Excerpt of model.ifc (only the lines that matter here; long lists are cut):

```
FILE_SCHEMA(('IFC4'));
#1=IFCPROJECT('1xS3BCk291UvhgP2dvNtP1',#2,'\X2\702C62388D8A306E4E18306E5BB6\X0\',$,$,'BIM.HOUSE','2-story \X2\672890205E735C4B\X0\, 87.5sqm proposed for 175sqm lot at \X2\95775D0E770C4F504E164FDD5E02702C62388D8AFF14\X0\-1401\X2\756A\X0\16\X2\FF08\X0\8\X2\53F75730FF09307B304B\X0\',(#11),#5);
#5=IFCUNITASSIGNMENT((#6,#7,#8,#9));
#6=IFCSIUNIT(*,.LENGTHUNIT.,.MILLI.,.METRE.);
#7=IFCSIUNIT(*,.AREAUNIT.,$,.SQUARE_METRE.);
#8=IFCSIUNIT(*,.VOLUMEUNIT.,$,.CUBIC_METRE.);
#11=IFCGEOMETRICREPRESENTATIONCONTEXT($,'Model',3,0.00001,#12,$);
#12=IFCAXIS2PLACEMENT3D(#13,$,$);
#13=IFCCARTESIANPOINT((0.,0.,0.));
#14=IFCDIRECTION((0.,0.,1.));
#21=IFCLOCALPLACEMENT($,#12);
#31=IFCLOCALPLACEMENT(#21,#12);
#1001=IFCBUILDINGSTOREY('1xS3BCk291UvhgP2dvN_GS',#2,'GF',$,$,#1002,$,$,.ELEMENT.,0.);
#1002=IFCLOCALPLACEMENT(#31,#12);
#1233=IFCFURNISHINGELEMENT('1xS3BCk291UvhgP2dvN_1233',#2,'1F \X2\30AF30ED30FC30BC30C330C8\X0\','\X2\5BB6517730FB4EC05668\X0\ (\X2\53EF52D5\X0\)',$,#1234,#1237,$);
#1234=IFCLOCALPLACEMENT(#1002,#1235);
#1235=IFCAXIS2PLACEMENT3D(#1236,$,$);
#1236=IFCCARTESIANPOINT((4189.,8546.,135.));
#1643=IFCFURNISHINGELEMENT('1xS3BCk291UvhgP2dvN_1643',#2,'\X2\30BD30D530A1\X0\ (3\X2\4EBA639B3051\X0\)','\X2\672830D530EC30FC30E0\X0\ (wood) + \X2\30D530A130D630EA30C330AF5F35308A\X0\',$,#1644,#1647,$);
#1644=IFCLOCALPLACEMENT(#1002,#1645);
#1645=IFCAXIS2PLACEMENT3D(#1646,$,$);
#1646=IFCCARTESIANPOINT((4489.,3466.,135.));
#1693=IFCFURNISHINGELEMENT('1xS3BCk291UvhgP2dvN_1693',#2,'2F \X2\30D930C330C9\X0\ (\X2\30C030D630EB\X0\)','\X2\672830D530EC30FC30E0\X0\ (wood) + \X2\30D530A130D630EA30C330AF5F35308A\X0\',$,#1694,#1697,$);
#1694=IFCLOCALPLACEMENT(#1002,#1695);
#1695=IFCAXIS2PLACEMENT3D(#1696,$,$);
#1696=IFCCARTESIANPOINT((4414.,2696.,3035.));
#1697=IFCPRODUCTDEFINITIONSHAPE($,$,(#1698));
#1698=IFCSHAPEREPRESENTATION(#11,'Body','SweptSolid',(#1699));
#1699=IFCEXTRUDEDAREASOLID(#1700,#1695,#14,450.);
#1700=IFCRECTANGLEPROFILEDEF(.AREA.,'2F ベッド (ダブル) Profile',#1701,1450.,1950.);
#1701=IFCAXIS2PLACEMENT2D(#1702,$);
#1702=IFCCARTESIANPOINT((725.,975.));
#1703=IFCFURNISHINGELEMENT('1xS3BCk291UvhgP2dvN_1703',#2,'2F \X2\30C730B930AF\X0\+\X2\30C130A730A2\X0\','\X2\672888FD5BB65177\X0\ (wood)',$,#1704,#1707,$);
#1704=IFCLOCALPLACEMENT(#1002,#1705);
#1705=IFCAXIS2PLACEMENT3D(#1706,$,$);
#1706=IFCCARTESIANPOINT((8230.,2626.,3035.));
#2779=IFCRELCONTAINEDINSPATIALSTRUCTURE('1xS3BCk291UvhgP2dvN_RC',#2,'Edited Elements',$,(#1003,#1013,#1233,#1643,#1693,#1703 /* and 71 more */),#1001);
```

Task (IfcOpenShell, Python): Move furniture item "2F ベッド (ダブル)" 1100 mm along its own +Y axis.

```python
import ifcopenshell
import ifcopenshell.api.geometry
import ifcopenshell.util.placement
import ifcopenshell.util.unit

model = ifcopenshell.open("model.ifc")
unit_scale = ifcopenshell.util.unit.calculate_unit_scale(model)

item = model.by_guid("1xS3BCk291UvhgP2dvN_1693")
matrix = ifcopenshell.util.placement.get_local_placement(item.ObjectPlacement)
matrix[:3, 3] += matrix[:3, 1] * 1.1 / unit_scale
ifcopenshell.api.geometry.edit_object_placement(model, product=item, matrix=matrix, is_si=False)

print(ifcopenshell.util.placement.get_local_placement(item.ObjectPlacement).round(3) + 0.0)

model.write("model_rev.ifc")
```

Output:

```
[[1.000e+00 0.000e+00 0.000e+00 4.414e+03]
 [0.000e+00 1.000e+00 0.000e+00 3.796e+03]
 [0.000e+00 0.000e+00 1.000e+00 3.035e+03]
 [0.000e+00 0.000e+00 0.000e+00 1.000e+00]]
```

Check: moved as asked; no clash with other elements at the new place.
